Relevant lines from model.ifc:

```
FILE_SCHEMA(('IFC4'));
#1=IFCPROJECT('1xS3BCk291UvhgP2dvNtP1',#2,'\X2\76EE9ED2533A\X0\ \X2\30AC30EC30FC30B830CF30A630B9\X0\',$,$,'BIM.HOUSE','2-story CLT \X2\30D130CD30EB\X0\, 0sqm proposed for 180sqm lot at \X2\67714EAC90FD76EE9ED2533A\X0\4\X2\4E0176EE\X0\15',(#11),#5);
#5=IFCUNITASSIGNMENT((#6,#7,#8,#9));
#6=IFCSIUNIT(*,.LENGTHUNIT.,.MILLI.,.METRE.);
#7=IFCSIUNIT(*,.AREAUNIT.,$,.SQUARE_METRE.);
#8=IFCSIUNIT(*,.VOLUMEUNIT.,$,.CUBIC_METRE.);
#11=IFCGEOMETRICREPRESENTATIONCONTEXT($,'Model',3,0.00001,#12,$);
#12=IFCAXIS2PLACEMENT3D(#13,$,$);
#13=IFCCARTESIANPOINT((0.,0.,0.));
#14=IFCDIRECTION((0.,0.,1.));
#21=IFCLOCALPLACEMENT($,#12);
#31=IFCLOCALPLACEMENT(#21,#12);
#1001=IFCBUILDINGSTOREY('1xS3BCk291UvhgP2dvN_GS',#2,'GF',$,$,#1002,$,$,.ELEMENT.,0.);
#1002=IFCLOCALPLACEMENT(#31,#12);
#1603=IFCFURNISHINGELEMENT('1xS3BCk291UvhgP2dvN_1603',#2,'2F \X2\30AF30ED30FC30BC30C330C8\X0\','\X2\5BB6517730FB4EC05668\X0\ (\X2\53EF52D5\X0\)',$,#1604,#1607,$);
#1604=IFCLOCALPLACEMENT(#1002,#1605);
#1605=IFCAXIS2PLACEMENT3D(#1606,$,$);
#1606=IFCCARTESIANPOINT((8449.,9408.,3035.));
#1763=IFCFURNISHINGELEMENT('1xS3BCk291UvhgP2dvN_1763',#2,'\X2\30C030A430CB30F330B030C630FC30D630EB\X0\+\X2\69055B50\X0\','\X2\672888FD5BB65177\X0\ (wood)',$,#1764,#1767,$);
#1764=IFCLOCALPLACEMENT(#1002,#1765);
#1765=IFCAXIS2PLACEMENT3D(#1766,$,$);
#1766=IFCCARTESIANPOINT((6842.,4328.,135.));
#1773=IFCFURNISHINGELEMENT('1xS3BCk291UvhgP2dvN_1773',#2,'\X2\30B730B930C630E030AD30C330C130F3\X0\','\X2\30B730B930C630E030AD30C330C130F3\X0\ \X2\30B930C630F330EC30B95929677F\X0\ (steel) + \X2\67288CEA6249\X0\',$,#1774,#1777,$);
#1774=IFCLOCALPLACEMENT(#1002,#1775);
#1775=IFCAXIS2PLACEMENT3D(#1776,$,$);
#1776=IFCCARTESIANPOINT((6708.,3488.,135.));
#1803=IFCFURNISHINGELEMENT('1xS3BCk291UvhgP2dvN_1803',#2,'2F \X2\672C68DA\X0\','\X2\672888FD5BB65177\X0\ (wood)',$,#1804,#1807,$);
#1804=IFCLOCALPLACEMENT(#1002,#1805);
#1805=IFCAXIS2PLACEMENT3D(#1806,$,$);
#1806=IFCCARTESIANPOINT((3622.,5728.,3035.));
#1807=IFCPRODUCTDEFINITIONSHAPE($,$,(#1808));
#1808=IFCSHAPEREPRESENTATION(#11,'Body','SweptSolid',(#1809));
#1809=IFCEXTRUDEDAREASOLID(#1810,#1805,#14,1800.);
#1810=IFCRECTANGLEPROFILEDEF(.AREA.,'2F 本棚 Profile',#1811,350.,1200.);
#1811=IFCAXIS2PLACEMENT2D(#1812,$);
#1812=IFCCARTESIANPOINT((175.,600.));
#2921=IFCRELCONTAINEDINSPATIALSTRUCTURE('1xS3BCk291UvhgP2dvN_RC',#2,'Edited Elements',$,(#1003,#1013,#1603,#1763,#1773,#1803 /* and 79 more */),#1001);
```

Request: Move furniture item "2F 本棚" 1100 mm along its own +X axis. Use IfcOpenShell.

```python
import ifcopenshell
import ifcopenshell.api.geometry
import ifcopenshell.util.placement
import ifcopenshell.util.unit

model = ifcopenshell.open("model.ifc")
unit_scale = ifcopenshell.util.unit.calculate_unit_scale(model)

item = model.by_id(1803)
matrix = ifcopenshell.util.placement.get_local_placement(item.ObjectPlacement)
matrix[:3, 3] += matrix[:3, 0] * 1.1 / unit_scale
ifcopenshell.api.geometry.edit_object_placement(model, product=item, matrix=matrix, is_si=False)

print(ifcopenshell.util.placement.get_local_placement(item.ObjectPlacement).round(3) + 0.0)

model.write("model_updated.ifc")
```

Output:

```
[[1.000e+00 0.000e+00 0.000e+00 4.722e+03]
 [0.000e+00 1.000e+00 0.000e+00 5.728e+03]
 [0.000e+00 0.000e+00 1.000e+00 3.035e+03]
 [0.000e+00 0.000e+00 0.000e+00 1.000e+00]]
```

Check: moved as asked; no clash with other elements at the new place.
